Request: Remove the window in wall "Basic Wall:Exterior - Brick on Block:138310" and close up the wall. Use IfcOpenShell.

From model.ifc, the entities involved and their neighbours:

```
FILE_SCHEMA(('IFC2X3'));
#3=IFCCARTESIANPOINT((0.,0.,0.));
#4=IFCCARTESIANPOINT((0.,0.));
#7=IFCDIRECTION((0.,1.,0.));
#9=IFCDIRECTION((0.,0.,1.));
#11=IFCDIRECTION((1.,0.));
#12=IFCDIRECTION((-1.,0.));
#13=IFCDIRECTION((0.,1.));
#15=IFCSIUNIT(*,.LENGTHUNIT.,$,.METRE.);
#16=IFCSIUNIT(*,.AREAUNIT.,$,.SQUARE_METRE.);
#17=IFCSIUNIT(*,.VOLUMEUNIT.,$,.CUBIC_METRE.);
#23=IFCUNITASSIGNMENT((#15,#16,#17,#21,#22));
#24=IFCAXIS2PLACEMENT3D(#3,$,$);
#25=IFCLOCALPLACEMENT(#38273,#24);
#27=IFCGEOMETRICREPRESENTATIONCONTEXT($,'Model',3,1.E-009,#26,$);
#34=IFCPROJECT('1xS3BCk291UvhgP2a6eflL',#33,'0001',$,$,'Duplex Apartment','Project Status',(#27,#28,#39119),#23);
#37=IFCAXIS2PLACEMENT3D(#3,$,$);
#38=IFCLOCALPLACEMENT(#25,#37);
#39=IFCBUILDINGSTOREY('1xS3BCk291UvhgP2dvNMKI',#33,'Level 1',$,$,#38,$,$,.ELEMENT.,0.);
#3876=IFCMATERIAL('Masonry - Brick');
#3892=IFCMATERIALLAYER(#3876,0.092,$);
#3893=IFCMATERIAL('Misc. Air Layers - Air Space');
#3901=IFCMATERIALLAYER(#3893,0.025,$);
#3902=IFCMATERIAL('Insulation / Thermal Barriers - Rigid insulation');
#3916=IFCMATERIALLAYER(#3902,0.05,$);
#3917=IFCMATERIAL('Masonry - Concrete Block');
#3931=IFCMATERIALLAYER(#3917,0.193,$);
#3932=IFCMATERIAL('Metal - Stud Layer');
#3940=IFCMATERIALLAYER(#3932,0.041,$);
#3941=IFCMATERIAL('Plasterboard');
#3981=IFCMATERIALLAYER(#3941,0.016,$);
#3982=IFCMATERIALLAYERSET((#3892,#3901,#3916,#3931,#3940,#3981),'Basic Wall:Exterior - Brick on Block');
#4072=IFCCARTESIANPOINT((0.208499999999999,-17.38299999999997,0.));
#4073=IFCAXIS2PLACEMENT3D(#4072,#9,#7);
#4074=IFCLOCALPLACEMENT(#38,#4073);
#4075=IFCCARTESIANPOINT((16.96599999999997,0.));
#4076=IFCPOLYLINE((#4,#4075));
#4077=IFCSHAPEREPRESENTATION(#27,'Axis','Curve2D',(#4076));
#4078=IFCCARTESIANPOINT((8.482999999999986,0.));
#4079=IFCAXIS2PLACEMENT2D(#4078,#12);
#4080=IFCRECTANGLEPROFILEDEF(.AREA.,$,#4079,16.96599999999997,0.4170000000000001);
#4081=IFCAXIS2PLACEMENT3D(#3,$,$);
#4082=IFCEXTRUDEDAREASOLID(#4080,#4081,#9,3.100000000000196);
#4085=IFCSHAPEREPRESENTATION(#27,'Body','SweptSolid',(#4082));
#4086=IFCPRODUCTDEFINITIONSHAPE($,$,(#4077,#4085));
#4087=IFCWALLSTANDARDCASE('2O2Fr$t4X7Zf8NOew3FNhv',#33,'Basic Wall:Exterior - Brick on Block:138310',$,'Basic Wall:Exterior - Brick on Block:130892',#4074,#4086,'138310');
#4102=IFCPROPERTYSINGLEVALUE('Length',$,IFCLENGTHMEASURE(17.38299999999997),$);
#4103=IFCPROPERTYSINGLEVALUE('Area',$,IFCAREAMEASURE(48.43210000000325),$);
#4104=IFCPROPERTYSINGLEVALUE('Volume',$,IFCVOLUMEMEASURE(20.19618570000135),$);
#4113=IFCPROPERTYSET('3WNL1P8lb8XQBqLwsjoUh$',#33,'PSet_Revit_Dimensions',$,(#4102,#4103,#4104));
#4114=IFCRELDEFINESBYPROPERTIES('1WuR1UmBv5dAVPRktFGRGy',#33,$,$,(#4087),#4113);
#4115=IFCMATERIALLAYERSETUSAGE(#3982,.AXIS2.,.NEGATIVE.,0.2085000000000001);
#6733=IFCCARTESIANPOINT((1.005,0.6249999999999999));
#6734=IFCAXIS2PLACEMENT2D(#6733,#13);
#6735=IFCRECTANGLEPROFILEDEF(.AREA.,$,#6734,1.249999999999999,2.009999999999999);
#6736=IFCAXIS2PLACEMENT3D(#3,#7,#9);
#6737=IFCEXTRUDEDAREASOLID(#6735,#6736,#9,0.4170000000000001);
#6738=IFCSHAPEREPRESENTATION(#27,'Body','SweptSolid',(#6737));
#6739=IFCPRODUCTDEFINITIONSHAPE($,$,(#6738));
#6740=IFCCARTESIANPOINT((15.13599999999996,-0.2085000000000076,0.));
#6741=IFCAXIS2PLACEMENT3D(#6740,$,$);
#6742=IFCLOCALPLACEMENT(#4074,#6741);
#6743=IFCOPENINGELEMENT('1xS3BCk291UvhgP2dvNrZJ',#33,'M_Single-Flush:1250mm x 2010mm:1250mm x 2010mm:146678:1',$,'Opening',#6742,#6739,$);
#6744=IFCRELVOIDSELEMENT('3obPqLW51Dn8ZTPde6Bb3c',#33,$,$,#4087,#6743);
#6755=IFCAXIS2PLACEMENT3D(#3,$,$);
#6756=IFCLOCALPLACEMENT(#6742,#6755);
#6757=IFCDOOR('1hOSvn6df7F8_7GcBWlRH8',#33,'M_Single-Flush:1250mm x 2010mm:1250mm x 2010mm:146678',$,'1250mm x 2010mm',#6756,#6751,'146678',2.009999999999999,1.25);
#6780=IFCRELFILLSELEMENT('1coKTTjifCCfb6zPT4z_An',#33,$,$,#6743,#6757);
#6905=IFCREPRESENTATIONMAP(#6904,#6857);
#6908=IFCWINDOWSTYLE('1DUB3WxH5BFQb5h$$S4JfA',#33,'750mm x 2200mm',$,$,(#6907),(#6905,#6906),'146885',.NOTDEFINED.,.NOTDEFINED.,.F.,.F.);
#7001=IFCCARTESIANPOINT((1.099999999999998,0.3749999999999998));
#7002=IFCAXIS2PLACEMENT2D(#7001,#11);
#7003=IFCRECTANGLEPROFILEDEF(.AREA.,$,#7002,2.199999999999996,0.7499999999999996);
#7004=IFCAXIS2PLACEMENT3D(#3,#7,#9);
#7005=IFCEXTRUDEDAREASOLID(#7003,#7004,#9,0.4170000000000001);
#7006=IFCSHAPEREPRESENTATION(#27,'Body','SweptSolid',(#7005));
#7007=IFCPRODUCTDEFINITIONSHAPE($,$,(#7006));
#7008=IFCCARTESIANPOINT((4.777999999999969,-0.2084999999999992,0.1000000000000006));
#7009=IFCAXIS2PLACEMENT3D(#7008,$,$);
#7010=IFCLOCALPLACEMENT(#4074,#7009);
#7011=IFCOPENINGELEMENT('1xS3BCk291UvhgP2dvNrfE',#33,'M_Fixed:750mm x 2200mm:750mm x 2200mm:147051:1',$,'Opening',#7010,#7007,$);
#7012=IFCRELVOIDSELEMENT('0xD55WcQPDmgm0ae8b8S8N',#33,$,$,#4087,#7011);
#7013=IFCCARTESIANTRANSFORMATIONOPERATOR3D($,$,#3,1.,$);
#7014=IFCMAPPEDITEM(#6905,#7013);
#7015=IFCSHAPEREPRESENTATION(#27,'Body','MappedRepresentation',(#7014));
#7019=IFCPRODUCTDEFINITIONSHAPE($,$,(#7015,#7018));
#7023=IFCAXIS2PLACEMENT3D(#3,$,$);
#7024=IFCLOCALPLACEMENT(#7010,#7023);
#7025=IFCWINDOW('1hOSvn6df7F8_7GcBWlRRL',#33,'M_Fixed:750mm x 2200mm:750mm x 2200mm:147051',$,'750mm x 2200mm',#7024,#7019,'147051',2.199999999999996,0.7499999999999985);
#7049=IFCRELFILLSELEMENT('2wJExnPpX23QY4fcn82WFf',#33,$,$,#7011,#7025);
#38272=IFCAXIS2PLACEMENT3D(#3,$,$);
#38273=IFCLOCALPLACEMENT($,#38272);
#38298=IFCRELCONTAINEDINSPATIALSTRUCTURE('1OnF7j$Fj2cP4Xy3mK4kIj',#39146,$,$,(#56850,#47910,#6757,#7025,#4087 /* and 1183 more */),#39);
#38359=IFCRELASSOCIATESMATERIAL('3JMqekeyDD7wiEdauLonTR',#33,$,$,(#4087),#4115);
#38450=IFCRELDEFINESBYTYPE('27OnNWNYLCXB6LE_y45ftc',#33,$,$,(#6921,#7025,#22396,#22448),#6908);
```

```python
import ifcopenshell
import ifcopenshell.api.feature
import ifcopenshell.api.pset
import ifcopenshell.api.root
import ifcopenshell.geom
import ifcopenshell.util.element
import ifcopenshell.util.shape
import ifcopenshell.util.unit

model = ifcopenshell.open("model.ifc")
area_scale = ifcopenshell.util.unit.calculate_unit_scale(model, "AREAUNIT")
volume_scale = ifcopenshell.util.unit.calculate_unit_scale(model, "VOLUMEUNIT")
settings = ifcopenshell.geom.settings()


def volume(element):
    """Net volume in cubic metres, openings subtracted."""
    shape = ifcopenshell.geom.create_shape(settings, element)
    return ifcopenshell.util.shape.get_volume(shape.geometry)


window = model.by_guid("1hOSvn6df7F8_7GcBWlRRL")
opening = window.FillsVoids[0].RelatingOpeningElement
wall = opening.VoidsElements[0].RelatingBuildingElement
before = volume(wall)

ifcopenshell.api.root.remove_product(model, product=window)
ifcopenshell.api.feature.remove_feature(model, feature=opening)

after = volume(wall)
thickness = 0.417  # wall thickness in metres

# Update the wall's stored quantities.
pset = model.by_id(ifcopenshell.util.element.get_pset(wall, "PSet_Revit_Dimensions", should_inherit=False)["id"])
ifcopenshell.api.pset.edit_pset(model, pset=pset, properties={
    "Area": model.create_entity("IfcAreaMeasure", after / thickness / area_scale),
    "Volume": model.create_entity("IfcVolumeMeasure", after / volume_scale),
})

print(f"wall volume {before:.3f} -> {after:.3f} m3")

model.write("model_updated.ifc")
```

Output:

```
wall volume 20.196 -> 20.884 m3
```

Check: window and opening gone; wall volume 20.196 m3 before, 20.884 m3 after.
